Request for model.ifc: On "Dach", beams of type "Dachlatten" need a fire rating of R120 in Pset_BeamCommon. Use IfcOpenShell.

First a look at what the model holds.

```python
import ifcopenshell
import ifcopenshell.util.element

model = ifcopenshell.open("model.ifc")
print(model.schema)
storey = next(s for s in model.by_type("IfcBuildingStorey") if s.Name == "Dach")
beams = [e for e in ifcopenshell.util.element.get_decomposition(storey) if e.is_a("IfcBeam")]
seen = {}
for e in beams:
    element_type = ifcopenshell.util.element.get_type(e)
    key = (element_type.Name if element_type != e and element_type else None, ifcopenshell.util.element.get_pset(e, "Pset_BeamCommon", "FireRating"))
    seen[key] = seen.get(key, 0) + 1
for (name, value), count in sorted(seen.items(), key=str):
    print(count, "x", name, "|", value)
```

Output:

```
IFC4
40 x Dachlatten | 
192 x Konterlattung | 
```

```python
import ifcopenshell
import ifcopenshell.api.pset
import ifcopenshell.util.element

model = ifcopenshell.open("model.ifc")

storey = next(s for s in model.by_type("IfcBuildingStorey") if s.Name == "Dach")
beams = [e for e in ifcopenshell.util.element.get_decomposition(storey) if e.is_a("IfcBeam")]

count = 0
for e in beams:
    element_type = ifcopenshell.util.element.get_type(e)
    if element_type in (None, e) or element_type.Name != "Dachlatten":
        continue
    # add_pset returns the element's existing set when there is one.
    pset = ifcopenshell.api.pset.add_pset(model, product=e, name="Pset_BeamCommon")
    ifcopenshell.api.pset.edit_pset(model, pset=pset, properties={"FireRating": "R120"})
    count += 1

print(count, "beams updated")

model.write("model_edited.ifc")
```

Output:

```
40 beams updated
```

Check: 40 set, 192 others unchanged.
